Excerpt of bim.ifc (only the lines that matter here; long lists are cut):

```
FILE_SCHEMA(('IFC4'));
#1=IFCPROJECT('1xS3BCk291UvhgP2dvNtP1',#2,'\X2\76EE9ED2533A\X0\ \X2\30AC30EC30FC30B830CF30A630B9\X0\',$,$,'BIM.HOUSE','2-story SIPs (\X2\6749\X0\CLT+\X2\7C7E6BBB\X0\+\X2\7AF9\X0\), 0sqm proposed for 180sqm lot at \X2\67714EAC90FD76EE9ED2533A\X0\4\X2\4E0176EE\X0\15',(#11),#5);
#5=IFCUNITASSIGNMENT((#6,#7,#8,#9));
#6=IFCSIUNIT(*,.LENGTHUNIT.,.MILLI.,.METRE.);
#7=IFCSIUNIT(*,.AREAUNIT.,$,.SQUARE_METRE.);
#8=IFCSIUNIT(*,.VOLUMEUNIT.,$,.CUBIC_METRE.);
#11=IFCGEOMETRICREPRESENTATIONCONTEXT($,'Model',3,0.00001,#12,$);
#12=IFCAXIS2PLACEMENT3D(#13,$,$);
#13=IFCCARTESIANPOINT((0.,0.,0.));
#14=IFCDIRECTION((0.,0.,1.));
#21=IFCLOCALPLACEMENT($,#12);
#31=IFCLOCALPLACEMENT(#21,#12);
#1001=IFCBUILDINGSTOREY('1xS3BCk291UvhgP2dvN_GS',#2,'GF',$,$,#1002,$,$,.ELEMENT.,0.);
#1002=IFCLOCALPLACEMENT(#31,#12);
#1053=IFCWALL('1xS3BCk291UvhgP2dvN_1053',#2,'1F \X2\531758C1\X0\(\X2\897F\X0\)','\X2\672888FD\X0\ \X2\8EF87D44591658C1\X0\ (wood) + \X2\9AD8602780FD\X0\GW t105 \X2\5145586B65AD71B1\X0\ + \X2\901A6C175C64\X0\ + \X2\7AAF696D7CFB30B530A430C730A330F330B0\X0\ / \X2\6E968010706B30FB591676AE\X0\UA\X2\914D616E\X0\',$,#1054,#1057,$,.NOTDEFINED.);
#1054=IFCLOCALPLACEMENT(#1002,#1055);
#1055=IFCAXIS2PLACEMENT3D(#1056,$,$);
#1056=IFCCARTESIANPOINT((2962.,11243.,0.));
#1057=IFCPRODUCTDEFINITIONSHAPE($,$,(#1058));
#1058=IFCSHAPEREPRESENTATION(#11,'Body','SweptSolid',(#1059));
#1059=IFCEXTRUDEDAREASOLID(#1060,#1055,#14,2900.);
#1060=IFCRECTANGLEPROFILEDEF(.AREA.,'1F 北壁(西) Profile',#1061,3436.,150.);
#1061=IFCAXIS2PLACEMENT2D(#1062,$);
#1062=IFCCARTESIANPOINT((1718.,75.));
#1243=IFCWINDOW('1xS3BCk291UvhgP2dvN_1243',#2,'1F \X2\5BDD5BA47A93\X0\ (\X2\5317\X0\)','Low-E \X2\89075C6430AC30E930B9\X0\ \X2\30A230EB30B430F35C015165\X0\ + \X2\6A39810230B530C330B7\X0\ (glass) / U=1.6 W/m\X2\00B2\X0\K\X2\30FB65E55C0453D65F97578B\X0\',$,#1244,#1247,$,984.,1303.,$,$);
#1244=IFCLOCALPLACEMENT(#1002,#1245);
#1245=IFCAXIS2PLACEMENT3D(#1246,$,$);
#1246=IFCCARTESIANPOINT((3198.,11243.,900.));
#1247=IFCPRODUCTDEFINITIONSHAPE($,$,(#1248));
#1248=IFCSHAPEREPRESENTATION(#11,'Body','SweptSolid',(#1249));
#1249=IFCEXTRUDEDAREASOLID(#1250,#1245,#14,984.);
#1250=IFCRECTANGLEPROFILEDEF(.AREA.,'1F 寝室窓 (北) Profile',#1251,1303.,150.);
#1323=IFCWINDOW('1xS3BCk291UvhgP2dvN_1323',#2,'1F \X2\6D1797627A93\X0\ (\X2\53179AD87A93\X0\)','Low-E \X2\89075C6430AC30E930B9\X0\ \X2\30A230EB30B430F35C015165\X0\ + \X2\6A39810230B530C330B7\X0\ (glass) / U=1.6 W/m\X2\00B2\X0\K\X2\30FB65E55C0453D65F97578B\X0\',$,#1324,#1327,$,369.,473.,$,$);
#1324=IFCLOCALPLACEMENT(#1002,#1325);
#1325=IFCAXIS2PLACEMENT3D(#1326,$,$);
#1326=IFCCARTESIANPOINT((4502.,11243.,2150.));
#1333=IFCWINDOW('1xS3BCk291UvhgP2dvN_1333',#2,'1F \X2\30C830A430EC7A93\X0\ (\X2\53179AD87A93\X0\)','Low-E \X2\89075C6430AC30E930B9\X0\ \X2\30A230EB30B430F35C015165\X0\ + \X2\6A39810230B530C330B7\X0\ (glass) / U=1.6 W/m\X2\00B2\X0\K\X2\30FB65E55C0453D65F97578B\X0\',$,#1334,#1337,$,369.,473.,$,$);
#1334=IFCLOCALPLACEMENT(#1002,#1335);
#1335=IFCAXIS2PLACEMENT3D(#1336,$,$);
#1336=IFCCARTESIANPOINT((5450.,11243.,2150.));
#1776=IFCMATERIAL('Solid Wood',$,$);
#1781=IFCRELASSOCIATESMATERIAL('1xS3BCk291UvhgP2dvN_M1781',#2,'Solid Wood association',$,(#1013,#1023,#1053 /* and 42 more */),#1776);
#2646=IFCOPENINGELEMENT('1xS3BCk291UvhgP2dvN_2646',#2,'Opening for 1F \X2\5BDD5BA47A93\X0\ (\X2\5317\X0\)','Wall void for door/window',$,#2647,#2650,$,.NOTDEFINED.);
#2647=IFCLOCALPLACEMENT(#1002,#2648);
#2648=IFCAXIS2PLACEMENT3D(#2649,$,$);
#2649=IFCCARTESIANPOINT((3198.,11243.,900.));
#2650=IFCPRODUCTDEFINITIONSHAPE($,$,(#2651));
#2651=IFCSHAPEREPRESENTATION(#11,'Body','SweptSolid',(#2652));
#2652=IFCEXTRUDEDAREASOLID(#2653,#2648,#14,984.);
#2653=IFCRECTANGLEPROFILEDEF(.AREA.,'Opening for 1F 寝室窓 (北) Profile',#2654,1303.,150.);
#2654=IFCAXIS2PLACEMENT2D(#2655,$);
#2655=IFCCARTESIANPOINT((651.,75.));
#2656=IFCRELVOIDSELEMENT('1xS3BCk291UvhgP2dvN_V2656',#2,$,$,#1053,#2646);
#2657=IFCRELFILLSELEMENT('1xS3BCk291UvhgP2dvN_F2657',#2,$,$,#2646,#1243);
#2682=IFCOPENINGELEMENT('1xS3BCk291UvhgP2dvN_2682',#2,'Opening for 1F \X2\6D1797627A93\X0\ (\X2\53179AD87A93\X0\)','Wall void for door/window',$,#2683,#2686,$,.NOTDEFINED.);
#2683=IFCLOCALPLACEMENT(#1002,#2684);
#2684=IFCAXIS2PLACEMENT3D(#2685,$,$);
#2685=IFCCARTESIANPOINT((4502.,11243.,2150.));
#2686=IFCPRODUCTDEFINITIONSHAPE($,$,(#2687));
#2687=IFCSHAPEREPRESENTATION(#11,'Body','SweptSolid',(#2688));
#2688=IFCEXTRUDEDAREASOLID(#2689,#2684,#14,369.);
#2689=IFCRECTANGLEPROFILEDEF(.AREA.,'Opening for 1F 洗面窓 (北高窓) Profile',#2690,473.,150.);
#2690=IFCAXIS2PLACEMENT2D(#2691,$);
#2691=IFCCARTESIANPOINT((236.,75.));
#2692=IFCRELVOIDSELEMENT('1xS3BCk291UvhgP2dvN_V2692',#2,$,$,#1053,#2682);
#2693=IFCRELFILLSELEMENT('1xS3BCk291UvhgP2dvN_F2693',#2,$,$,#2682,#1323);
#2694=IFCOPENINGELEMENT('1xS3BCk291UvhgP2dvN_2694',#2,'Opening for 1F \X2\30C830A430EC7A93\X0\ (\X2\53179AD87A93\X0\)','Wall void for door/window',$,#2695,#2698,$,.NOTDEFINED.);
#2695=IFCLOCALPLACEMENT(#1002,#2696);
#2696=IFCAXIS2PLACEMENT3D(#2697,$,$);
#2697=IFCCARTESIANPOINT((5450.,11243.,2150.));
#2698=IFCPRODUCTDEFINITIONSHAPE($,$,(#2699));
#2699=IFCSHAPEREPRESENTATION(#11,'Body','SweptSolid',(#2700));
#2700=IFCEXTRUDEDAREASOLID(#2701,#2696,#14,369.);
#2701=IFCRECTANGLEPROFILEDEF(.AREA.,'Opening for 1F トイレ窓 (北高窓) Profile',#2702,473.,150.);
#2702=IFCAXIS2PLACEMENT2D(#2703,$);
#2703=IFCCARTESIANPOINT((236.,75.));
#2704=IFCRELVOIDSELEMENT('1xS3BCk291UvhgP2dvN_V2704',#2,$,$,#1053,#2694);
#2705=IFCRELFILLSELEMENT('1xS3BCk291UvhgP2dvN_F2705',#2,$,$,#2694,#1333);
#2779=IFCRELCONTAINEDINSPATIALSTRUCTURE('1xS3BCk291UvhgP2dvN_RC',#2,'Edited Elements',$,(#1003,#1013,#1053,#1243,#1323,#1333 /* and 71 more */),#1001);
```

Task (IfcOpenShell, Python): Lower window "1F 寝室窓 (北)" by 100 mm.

```python
import numpy as np
import ifcopenshell
import ifcopenshell.api.geometry
import ifcopenshell.util.placement
import ifcopenshell.util.unit

model = ifcopenshell.open("bim.ifc")
unit_scale = ifcopenshell.util.unit.calculate_unit_scale(model)

window = model.by_id(1243)
opening = window.FillsVoids[0].RelatingOpeningElement
dz = -100.0

shift = np.array([0.0, 0.0, dz])
# The window is not placed relative to its opening, so move both.
for product in (opening, window):
    matrix = ifcopenshell.util.placement.get_local_placement(product.ObjectPlacement)
    matrix[:3, 3] += shift
    ifcopenshell.api.geometry.edit_object_placement(model, product=product, matrix=matrix, is_si=False)

print(f"moved by {dz * unit_scale:+.3f} m")

model.write("bim_edited.ifc")
```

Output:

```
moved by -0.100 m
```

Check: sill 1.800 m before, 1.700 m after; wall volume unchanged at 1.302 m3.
